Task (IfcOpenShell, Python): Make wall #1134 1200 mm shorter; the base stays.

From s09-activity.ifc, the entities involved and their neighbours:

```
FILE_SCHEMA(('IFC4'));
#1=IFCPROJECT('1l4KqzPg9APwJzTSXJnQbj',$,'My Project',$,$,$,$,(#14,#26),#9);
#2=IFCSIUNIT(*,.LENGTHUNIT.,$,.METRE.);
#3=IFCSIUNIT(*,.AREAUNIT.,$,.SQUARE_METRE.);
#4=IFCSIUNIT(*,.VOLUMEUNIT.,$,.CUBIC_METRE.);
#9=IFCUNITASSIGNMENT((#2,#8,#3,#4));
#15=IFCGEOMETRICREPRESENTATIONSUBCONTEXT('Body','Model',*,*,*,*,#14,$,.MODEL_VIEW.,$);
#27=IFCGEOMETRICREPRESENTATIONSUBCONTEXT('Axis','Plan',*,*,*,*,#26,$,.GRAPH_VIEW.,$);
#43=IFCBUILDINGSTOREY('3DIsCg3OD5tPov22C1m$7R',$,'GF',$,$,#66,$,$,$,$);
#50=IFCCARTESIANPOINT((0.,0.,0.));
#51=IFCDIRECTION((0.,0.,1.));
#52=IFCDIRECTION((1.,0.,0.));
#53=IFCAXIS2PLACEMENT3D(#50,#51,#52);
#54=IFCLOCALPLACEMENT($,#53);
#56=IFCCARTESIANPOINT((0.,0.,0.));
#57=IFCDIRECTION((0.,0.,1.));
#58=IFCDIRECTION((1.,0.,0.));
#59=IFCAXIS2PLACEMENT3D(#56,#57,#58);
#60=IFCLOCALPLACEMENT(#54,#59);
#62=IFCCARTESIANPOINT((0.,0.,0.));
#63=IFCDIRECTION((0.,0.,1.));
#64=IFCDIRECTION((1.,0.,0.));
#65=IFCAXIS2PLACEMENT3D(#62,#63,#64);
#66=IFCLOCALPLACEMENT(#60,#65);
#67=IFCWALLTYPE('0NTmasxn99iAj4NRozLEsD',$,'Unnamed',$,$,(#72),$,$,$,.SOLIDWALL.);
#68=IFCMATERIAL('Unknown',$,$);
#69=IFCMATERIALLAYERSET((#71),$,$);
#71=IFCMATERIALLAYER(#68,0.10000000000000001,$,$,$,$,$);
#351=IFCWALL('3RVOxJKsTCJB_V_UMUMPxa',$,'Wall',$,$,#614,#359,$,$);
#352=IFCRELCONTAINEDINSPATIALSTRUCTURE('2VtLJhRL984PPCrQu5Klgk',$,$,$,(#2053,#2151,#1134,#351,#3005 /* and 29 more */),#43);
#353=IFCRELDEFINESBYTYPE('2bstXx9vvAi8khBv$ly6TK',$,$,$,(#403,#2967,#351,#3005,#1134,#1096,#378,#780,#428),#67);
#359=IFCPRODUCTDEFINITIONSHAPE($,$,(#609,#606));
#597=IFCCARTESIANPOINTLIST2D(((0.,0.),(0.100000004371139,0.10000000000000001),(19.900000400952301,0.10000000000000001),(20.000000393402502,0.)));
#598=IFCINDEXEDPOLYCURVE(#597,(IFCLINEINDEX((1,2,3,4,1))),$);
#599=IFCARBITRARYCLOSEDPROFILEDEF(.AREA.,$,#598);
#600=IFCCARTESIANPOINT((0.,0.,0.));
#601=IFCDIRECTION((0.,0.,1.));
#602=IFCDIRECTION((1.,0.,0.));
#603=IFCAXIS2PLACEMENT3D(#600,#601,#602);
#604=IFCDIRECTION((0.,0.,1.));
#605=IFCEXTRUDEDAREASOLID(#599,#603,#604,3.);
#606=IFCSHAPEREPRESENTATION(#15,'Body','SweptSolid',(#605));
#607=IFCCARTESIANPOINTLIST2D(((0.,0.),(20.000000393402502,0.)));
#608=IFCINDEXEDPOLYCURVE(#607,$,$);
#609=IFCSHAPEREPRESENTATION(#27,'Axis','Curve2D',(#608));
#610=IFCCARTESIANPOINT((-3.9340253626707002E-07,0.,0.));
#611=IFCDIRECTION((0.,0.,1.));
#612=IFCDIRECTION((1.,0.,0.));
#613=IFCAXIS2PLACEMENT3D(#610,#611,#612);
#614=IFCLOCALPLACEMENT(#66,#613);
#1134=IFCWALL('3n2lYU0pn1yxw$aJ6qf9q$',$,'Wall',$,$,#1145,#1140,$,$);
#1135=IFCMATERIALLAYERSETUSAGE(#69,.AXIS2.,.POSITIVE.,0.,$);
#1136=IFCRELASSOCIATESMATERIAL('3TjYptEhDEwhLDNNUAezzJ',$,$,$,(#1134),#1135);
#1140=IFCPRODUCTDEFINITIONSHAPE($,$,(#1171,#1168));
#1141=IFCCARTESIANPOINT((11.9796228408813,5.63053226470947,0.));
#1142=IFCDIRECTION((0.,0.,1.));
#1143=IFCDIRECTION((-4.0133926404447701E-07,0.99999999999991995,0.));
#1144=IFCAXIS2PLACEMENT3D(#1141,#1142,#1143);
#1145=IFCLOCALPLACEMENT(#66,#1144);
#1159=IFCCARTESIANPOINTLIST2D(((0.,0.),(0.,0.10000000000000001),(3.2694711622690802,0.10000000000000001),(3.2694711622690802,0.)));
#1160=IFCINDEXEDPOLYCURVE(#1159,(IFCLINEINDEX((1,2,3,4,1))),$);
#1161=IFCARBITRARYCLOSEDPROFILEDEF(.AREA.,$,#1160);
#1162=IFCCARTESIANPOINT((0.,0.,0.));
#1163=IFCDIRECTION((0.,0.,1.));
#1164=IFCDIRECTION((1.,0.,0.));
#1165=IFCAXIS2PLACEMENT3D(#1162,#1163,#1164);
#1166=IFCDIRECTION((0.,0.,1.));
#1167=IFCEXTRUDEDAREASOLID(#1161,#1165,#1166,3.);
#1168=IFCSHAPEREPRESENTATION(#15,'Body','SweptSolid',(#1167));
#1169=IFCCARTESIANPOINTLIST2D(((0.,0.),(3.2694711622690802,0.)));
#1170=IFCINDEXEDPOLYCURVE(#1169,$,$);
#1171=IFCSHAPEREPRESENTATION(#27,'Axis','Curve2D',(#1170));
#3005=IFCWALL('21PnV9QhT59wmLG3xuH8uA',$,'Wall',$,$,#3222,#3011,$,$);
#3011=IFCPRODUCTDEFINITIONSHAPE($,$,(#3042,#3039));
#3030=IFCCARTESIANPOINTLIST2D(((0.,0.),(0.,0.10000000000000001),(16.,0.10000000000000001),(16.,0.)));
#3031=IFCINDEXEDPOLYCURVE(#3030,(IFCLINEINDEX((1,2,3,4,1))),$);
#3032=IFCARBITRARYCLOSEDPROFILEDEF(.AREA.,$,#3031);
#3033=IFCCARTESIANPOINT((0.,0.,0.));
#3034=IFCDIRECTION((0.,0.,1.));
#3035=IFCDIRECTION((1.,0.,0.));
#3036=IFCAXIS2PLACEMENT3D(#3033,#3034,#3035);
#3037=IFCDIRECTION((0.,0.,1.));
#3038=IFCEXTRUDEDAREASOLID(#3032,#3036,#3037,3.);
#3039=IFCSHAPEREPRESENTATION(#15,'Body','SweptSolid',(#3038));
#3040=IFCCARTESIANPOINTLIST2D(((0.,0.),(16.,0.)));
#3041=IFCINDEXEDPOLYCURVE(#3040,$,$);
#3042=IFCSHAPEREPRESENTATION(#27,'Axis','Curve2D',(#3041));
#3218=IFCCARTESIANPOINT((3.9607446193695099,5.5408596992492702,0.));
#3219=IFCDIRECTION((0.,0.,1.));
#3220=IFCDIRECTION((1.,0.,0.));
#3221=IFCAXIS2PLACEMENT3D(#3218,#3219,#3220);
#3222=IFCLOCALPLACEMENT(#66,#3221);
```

```python
import ifcopenshell
import ifcopenshell.geom
import ifcopenshell.util.representation
import ifcopenshell.util.shape
import ifcopenshell.util.unit

model = ifcopenshell.open("s09-activity.ifc")
unit_scale = ifcopenshell.util.unit.calculate_unit_scale(model)
settings = ifcopenshell.geom.settings()


def volume(element):
    """Net volume in cubic metres, openings subtracted."""
    shape = ifcopenshell.geom.create_shape(settings, element)
    return ifcopenshell.util.shape.get_volume(shape.geometry)


wall = model.by_guid("3n2lYU0pn1yxw$aJ6qf9q$")
before = volume(wall)

body = ifcopenshell.util.representation.get_representation(wall, "Model", "Body")
solid = body.Items[0]
old_height = solid.Depth
solid.Depth -= 1.2 / unit_scale
after = volume(wall)

print(f"height {old_height:g} -> {solid.Depth:g}, volume {before:.3f} -> {after:.3f} m3")

model.write("s09-activity_updated.ifc")
```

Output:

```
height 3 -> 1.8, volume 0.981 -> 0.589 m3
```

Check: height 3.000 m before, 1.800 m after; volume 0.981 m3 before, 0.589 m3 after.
